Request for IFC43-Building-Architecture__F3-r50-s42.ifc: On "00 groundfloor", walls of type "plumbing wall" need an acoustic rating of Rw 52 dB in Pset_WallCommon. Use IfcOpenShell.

First a look at what the model holds.

```python
import ifcopenshell
import ifcopenshell.util.element

model = ifcopenshell.open("IFC43-Building-Architecture__F3-r50-s42.ifc")
print(model.schema)
storey = next(s for s in model.by_type("IfcBuildingStorey") if s.Name == "00 groundfloor")
walls = [e for e in ifcopenshell.util.element.get_decomposition(storey) if e.is_a("IfcWall")]
seen = {}
for e in walls:
    element_type = ifcopenshell.util.element.get_type(e)
    key = (element_type.Name if element_type != e and element_type else None, ifcopenshell.util.element.get_pset(e, "Pset_WallCommon", "AcousticRating"))
    seen[key] = seen.get(key, 0) + 1
for (name, value), count in sorted(seen.items(), key=str):
    print(count, "x", name, "|", value)
```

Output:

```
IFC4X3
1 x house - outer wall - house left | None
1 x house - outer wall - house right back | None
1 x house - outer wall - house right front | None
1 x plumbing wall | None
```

```python
import ifcopenshell
import ifcopenshell.api.pset
import ifcopenshell.util.element

model = ifcopenshell.open("IFC43-Building-Architecture__F3-r50-s42.ifc")

storey = next(s for s in model.by_type("IfcBuildingStorey") if s.Name == "00 groundfloor")
walls = [e for e in ifcopenshell.util.element.get_decomposition(storey) if e.is_a("IfcWall")]

count = 0
for e in walls:
    element_type = ifcopenshell.util.element.get_type(e)
    if element_type in (None, e) or element_type.Name != "plumbing wall":
        continue
    # add_pset returns the element's existing set when there is one.
    pset = ifcopenshell.api.pset.add_pset(model, product=e, name="Pset_WallCommon")
    ifcopenshell.api.pset.edit_pset(model, pset=pset, properties={"AcousticRating": "Rw 52 dB"})
    count += 1

print(count, "walls updated")

model.write("IFC43-Building-Architecture__F3-r50-s42_edited.ifc")
```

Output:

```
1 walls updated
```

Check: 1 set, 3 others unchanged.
